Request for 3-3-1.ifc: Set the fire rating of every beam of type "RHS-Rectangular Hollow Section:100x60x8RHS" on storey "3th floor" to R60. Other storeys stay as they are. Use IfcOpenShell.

First a look at what the model holds.

```python
import ifcopenshell
import ifcopenshell.util.element

model = ifcopenshell.open("3-3-1.ifc")
print(model.schema)
storey = next(s for s in model.by_type("IfcBuildingStorey") if s.Name == "3th floor")
beams = [e for e in ifcopenshell.util.element.get_decomposition(storey) if e.is_a("IfcBeam")]
seen = {}
for e in beams:
    element_type = ifcopenshell.util.element.get_type(e)
    key = (element_type.Name if element_type != e and element_type else None, ifcopenshell.util.element.get_pset(e, "Pset_BeamCommon", "FireRating"))
    seen[key] = seen.get(key, 0) + 1
for (name, value), count in sorted(seen.items(), key=str):
    print(count, "x", name, "|", value)
```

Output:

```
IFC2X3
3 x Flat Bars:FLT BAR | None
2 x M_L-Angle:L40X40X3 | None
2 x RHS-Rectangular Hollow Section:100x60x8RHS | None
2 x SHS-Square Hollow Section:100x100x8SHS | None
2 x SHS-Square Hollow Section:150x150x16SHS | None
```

```python
import ifcopenshell
import ifcopenshell.api.pset
import ifcopenshell.util.element

model = ifcopenshell.open("3-3-1.ifc")

storey = next(s for s in model.by_type("IfcBuildingStorey") if s.Name == "3th floor")
beams = [e for e in ifcopenshell.util.element.get_decomposition(storey) if e.is_a("IfcBeam")]

count = 0
for e in beams:
    element_type = ifcopenshell.util.element.get_type(e)
    if element_type in (None, e) or element_type.Name != "RHS-Rectangular Hollow Section:100x60x8RHS":
        continue
    # add_pset returns the element's existing set when there is one.
    pset = ifcopenshell.api.pset.add_pset(model, product=e, name="Pset_BeamCommon")
    ifcopenshell.api.pset.edit_pset(model, pset=pset, properties={"FireRating": "R60"})
    count += 1

print(count, "beams updated")

model.write("3-3-1_v2.ifc")
```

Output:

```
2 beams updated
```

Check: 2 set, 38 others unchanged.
